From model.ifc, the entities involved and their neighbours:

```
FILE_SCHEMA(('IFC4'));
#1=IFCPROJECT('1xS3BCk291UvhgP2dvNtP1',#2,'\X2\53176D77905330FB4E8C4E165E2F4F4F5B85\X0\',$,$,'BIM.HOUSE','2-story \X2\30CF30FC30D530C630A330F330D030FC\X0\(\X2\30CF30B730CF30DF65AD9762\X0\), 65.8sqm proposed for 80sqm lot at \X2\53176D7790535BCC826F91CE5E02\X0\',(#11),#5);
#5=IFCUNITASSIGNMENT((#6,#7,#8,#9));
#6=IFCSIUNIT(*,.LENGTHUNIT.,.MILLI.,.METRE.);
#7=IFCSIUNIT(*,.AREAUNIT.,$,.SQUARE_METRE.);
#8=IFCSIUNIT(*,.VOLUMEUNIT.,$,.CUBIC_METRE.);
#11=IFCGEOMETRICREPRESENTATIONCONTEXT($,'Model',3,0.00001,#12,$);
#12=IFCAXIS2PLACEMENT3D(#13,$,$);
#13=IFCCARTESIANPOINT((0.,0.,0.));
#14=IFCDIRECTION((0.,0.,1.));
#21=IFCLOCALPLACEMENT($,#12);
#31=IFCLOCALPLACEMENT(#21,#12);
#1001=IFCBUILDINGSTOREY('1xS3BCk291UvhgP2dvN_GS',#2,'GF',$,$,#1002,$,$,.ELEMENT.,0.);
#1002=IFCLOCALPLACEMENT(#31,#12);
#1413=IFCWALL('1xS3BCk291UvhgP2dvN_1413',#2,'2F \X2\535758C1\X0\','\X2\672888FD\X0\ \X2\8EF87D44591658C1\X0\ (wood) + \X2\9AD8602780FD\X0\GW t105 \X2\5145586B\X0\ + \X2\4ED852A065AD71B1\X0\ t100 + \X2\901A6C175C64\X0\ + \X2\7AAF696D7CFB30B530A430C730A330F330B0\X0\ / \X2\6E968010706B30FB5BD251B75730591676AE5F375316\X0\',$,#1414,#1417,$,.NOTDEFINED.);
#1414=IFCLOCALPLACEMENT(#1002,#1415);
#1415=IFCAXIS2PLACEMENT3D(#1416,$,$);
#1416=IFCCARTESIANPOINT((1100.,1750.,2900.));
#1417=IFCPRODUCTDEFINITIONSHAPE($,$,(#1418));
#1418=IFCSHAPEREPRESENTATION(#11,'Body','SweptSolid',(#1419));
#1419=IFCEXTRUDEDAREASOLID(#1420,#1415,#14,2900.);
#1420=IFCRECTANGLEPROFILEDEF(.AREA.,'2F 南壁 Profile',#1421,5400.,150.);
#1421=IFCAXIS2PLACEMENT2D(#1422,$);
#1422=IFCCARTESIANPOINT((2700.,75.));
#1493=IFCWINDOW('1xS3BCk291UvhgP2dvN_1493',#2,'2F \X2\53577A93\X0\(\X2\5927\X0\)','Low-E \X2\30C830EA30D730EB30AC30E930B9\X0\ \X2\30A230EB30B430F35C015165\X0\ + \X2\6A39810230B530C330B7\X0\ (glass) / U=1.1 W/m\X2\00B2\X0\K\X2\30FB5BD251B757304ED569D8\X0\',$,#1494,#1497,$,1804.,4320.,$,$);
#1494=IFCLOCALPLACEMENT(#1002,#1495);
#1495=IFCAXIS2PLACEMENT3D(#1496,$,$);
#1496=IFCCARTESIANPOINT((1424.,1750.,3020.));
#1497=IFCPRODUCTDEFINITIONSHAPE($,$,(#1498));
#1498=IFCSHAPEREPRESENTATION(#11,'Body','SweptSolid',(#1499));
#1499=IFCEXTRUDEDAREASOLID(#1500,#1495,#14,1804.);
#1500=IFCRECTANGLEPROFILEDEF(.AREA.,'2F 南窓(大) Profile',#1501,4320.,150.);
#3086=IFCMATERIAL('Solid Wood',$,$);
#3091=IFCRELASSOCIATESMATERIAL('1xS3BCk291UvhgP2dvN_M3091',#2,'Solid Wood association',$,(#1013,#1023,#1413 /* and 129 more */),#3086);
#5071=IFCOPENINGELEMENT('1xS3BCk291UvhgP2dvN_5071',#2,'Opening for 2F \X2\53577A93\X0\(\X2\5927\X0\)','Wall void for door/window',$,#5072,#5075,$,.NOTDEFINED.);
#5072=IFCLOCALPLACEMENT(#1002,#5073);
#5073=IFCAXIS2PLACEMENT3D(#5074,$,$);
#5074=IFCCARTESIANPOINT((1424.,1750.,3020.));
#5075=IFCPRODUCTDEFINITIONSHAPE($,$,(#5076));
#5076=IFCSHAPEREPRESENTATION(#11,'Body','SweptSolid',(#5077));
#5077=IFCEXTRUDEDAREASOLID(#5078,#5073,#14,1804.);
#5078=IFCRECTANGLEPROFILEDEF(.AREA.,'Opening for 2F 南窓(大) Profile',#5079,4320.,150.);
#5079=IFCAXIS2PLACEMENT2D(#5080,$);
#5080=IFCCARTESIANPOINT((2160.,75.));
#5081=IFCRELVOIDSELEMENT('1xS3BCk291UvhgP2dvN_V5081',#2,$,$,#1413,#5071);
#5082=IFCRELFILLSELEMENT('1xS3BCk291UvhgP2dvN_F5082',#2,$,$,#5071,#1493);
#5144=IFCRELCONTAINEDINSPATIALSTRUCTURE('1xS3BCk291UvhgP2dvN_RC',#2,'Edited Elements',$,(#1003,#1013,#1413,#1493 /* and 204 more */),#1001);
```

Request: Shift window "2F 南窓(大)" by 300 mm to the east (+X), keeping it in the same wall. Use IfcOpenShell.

```python
import ifcopenshell
import ifcopenshell.api.geometry
import ifcopenshell.util.placement
import ifcopenshell.util.unit

model = ifcopenshell.open("model.ifc")
unit_scale = ifcopenshell.util.unit.calculate_unit_scale(model)

window = model.by_id(1493)
opening = window.FillsVoids[0].RelatingOpeningElement
wall = opening.VoidsElements[0].RelatingBuildingElement

wall_matrix = ifcopenshell.util.placement.get_local_placement(wall.ObjectPlacement)
shift = wall_matrix[:3, 0] * 0.3 / unit_scale
before = ifcopenshell.util.placement.get_local_placement(window.ObjectPlacement)[:3, 3].copy()

# The window is not placed relative to its opening, so move both.
for product in (opening, window):
    matrix = ifcopenshell.util.placement.get_local_placement(product.ObjectPlacement)
    matrix[:3, 3] += shift
    ifcopenshell.api.geometry.edit_object_placement(model, product=product, matrix=matrix, is_si=False)

after = ifcopenshell.util.placement.get_local_placement(window.ObjectPlacement)[:3, 3]
print("window moved by", (after - before).round(3) + 0.0)

model.write("model_v2.ifc")
```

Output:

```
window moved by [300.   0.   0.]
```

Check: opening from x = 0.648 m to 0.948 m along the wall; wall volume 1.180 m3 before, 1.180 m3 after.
